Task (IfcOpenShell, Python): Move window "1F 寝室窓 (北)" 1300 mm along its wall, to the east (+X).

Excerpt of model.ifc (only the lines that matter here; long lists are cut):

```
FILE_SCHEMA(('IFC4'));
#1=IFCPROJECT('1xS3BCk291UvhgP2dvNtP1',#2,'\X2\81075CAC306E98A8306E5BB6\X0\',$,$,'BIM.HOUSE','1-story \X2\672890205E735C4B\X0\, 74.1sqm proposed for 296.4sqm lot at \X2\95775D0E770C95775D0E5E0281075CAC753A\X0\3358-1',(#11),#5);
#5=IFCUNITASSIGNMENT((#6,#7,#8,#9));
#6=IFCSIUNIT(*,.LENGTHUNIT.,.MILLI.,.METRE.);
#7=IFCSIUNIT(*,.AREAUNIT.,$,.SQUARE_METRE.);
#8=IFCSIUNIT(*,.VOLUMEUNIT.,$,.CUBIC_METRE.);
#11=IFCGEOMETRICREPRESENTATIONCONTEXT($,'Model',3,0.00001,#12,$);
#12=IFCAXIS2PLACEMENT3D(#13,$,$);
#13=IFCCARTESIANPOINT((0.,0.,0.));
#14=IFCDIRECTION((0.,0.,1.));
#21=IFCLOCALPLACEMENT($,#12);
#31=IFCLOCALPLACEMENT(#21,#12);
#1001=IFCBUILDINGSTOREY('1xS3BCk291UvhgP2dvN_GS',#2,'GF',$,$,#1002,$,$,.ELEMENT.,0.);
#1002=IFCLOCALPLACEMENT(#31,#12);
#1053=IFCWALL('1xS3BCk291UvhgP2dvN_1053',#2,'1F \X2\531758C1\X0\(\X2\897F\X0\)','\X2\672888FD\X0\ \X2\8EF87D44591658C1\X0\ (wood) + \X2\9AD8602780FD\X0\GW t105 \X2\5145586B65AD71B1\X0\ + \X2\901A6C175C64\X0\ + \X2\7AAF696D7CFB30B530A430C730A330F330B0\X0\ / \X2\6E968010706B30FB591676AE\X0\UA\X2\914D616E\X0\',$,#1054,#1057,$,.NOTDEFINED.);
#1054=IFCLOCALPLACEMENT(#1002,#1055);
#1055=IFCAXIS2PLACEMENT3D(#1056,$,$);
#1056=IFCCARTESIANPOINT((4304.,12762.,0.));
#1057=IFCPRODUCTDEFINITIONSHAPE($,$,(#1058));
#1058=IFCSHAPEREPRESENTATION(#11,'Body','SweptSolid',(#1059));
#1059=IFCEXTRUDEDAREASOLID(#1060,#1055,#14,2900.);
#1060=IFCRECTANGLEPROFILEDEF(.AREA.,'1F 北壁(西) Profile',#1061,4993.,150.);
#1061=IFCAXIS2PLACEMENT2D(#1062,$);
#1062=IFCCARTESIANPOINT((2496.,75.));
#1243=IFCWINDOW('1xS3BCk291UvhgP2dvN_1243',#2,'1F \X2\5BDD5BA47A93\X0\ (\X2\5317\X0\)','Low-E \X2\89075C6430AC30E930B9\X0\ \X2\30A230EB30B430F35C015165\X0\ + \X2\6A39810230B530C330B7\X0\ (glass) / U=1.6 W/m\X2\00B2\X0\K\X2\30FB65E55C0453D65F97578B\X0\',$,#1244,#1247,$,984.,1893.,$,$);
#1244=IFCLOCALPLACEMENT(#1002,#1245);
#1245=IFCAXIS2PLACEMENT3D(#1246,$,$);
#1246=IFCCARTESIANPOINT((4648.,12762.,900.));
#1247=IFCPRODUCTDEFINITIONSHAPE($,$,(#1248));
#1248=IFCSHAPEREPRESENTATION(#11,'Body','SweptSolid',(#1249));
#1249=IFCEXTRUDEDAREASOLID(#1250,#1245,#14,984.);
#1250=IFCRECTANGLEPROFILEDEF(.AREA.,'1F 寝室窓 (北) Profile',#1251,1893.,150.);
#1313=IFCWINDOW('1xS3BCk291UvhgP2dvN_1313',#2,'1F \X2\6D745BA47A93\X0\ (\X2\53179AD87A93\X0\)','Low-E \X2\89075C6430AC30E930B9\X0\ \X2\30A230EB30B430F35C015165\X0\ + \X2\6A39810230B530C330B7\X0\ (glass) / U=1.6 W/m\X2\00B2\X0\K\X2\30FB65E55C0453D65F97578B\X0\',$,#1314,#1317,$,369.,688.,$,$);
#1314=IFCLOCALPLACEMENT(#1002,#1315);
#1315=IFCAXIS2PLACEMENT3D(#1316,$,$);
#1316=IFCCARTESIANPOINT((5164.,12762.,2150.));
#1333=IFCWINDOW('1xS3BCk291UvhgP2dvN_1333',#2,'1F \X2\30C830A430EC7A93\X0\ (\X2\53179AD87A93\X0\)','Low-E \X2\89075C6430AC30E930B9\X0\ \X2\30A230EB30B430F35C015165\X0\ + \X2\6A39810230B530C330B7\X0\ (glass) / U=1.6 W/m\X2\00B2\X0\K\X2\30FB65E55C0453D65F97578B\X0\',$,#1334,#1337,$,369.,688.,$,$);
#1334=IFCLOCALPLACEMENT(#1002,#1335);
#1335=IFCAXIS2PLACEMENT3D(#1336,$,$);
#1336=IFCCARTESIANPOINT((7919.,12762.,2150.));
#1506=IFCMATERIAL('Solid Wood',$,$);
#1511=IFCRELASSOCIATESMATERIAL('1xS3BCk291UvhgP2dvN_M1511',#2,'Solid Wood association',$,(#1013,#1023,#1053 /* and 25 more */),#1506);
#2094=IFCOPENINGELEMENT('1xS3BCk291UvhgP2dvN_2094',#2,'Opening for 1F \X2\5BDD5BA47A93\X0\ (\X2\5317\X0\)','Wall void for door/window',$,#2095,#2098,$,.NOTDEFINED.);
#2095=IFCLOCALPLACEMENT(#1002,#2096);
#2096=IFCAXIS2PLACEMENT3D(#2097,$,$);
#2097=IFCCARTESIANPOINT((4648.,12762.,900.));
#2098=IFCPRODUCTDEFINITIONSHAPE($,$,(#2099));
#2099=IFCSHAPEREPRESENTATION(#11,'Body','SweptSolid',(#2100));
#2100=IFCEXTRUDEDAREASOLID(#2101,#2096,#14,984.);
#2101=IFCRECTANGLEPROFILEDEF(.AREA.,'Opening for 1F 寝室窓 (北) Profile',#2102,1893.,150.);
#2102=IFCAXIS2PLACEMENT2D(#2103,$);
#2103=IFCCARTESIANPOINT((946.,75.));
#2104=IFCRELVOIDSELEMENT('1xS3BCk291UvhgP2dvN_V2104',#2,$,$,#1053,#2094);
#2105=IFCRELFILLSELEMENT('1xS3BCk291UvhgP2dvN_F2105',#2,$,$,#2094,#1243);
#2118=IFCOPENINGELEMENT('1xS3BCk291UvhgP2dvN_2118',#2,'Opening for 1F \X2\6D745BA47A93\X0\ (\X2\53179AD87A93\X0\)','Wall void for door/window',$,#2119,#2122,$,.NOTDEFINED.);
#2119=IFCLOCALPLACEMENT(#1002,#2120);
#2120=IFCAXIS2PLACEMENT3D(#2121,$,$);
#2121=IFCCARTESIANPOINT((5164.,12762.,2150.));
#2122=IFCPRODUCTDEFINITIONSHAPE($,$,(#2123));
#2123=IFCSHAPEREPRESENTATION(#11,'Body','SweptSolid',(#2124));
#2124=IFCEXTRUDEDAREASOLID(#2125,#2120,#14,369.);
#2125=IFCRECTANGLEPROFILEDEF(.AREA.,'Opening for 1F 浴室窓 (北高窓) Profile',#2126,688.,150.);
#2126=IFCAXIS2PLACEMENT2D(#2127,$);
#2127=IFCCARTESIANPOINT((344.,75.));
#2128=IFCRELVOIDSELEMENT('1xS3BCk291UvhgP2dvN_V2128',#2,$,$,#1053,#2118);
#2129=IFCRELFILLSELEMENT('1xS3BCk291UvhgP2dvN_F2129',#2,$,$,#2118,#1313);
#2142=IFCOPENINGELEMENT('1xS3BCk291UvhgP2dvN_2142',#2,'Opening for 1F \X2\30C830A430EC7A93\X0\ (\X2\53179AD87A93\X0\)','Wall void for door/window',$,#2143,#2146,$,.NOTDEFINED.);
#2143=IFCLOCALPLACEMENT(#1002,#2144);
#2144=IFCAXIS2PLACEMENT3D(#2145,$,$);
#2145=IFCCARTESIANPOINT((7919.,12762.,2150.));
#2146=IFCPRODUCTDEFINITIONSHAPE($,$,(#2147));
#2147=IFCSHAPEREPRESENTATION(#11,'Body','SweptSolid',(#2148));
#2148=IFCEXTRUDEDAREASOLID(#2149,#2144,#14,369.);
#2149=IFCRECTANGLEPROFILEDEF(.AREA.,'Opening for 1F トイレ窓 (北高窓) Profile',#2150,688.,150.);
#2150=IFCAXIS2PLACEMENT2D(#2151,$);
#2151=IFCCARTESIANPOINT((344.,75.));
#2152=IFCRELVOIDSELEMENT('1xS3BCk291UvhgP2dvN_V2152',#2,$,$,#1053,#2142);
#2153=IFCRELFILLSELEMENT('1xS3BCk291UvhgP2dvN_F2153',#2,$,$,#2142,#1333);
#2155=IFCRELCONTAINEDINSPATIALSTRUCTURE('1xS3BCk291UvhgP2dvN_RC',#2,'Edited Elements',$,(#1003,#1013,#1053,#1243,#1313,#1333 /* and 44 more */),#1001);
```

```python
import ifcopenshell
import ifcopenshell.api.geometry
import ifcopenshell.util.placement
import ifcopenshell.util.unit

model = ifcopenshell.open("model.ifc")
unit_scale = ifcopenshell.util.unit.calculate_unit_scale(model)

window = model.by_guid("1xS3BCk291UvhgP2dvN_1243")
opening = window.FillsVoids[0].RelatingOpeningElement
wall = opening.VoidsElements[0].RelatingBuildingElement

wall_matrix = ifcopenshell.util.placement.get_local_placement(wall.ObjectPlacement)
shift = wall_matrix[:3, 0] * 1.3 / unit_scale
before = ifcopenshell.util.placement.get_local_placement(window.ObjectPlacement)[:3, 3].copy()

# The window is not placed relative to its opening, so move both.
for product in (opening, window):
    matrix = ifcopenshell.util.placement.get_local_placement(product.ObjectPlacement)
    matrix[:3, 3] += shift
    ifcopenshell.api.geometry.edit_object_placement(model, product=product, matrix=matrix, is_si=False)

after = ifcopenshell.util.placement.get_local_placement(window.ObjectPlacement)[:3, 3]
print("window moved by", (after - before).round(3) + 0.0)

model.write("model_v2.ifc")
```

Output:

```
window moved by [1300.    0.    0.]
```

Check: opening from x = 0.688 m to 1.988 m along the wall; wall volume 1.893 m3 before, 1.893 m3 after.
